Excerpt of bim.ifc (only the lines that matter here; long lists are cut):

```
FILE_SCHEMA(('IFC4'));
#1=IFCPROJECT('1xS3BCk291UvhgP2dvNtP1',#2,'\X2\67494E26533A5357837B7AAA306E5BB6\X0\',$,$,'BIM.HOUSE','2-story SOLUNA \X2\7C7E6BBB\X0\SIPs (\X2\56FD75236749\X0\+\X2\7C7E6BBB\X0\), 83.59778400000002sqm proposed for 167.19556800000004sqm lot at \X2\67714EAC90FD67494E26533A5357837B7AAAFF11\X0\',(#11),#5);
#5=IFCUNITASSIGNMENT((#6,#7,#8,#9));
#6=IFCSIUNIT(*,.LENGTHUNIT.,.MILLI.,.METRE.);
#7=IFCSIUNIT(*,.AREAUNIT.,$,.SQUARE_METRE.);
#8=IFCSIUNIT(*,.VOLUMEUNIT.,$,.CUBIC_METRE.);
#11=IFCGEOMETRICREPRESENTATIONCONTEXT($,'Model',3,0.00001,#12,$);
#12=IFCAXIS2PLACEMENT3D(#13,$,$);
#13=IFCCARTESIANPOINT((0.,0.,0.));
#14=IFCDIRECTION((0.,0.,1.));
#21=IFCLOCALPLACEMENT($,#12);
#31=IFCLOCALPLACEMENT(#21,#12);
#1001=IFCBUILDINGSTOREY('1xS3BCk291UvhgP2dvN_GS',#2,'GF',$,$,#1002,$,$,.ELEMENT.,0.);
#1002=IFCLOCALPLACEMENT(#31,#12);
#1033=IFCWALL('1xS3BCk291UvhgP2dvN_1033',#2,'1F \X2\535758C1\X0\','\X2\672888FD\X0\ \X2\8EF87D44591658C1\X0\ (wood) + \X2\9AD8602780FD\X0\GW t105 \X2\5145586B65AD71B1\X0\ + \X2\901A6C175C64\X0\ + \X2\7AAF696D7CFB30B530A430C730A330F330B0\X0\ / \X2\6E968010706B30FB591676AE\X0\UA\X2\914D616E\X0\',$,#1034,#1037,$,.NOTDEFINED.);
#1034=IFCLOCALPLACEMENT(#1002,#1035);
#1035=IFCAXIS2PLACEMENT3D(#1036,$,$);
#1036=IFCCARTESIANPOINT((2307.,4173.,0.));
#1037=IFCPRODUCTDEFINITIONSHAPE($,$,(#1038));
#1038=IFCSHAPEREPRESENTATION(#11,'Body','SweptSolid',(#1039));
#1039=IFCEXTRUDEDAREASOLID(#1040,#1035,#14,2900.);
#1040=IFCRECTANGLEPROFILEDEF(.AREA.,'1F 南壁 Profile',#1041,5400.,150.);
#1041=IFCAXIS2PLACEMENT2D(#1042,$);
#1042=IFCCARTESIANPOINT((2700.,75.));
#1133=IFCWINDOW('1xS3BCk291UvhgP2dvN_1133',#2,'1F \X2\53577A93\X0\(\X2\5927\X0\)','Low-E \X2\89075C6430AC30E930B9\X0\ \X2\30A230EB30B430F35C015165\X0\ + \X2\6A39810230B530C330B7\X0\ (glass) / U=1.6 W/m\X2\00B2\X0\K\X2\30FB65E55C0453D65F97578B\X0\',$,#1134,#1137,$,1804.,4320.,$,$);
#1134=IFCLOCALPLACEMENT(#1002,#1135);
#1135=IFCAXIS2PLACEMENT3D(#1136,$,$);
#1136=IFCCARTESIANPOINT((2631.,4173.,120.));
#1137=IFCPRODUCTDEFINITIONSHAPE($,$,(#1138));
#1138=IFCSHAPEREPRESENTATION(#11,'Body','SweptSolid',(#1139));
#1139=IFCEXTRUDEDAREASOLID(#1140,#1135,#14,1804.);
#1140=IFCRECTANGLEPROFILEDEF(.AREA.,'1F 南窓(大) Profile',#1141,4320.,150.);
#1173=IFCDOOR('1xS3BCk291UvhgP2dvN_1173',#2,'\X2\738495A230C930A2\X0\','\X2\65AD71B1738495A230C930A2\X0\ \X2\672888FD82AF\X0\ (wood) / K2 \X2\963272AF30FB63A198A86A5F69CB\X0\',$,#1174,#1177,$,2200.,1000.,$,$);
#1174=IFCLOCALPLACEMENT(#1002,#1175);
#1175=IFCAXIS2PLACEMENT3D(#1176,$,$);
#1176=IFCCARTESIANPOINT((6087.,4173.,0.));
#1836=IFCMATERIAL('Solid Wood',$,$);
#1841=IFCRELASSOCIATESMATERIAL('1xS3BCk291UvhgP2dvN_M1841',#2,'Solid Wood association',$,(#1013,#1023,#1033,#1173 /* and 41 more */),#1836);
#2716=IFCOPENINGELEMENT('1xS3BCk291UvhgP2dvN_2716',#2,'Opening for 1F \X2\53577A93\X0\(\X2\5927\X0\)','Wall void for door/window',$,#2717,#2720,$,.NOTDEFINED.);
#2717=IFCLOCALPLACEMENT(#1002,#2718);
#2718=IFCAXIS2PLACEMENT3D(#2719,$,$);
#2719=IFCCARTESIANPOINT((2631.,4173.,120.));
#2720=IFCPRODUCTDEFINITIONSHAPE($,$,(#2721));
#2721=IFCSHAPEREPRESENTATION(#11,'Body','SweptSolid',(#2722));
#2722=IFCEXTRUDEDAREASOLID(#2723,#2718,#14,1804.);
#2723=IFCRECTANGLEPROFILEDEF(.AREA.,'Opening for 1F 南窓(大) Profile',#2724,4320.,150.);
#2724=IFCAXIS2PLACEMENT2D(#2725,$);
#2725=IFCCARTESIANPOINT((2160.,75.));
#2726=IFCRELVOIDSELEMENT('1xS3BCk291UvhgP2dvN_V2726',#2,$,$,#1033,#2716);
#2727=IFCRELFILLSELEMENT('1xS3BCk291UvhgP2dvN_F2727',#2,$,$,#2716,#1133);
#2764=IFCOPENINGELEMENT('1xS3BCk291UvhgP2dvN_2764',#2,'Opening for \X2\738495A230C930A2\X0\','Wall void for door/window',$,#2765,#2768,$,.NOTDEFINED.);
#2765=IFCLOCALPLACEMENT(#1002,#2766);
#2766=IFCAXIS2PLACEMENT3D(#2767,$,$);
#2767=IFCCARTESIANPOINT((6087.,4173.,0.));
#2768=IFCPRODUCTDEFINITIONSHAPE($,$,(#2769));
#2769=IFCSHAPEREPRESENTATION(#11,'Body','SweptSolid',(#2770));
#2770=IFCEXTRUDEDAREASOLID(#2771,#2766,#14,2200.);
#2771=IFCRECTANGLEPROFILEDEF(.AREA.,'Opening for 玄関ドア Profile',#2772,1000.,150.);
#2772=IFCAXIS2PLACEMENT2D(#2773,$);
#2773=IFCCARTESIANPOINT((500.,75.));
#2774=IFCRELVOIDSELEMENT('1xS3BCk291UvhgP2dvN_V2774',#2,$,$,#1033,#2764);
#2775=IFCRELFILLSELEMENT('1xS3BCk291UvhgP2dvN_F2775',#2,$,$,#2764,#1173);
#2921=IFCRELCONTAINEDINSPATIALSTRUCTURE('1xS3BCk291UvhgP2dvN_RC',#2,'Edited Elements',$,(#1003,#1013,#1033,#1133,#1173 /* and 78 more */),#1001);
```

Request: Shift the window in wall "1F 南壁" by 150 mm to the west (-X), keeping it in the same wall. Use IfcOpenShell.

```python
import ifcopenshell
import ifcopenshell.api.geometry
import ifcopenshell.util.placement
import ifcopenshell.util.unit

model = ifcopenshell.open("bim.ifc")
unit_scale = ifcopenshell.util.unit.calculate_unit_scale(model)

window = model.by_guid("1xS3BCk291UvhgP2dvN_1133")
opening = window.FillsVoids[0].RelatingOpeningElement
wall = opening.VoidsElements[0].RelatingBuildingElement

wall_matrix = ifcopenshell.util.placement.get_local_placement(wall.ObjectPlacement)
shift = wall_matrix[:3, 0] * -0.15 / unit_scale
before = ifcopenshell.util.placement.get_local_placement(window.ObjectPlacement)[:3, 3].copy()

# The window is not placed relative to its opening, so move both.
for product in (opening, window):
    matrix = ifcopenshell.util.placement.get_local_placement(product.ObjectPlacement)
    matrix[:3, 3] += shift
    ifcopenshell.api.geometry.edit_object_placement(model, product=product, matrix=matrix, is_si=False)

after = ifcopenshell.util.placement.get_local_placement(window.ObjectPlacement)[:3, 3]
print("window moved by", (after - before).round(3) + 0.0)

model.write("bim_edited.ifc")
```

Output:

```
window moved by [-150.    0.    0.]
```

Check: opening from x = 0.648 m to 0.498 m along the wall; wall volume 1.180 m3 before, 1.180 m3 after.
